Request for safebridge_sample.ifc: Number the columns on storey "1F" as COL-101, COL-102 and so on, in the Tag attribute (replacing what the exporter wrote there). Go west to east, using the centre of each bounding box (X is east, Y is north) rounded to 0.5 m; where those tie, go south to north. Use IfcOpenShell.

First a look at what the model holds.

```python
import ifcopenshell
import ifcopenshell.util.element
import ifcopenshell.util.placement

model = ifcopenshell.open("safebridge_sample.ifc")
print(model.schema)
storey = next(s for s in model.by_type("IfcBuildingStorey") if s.Name == "1F")
columns = [e for e in ifcopenshell.util.element.get_decomposition(storey) if e.is_a("IfcColumn")]
for e in sorted(columns, key=lambda e: e.id()):
    origin = ifcopenshell.util.placement.get_local_placement(e.ObjectPlacement)[:3, 3]
    print(e.id(), e.Tag, e.Name, origin.round(2) + 0.0, sep=" | ")
```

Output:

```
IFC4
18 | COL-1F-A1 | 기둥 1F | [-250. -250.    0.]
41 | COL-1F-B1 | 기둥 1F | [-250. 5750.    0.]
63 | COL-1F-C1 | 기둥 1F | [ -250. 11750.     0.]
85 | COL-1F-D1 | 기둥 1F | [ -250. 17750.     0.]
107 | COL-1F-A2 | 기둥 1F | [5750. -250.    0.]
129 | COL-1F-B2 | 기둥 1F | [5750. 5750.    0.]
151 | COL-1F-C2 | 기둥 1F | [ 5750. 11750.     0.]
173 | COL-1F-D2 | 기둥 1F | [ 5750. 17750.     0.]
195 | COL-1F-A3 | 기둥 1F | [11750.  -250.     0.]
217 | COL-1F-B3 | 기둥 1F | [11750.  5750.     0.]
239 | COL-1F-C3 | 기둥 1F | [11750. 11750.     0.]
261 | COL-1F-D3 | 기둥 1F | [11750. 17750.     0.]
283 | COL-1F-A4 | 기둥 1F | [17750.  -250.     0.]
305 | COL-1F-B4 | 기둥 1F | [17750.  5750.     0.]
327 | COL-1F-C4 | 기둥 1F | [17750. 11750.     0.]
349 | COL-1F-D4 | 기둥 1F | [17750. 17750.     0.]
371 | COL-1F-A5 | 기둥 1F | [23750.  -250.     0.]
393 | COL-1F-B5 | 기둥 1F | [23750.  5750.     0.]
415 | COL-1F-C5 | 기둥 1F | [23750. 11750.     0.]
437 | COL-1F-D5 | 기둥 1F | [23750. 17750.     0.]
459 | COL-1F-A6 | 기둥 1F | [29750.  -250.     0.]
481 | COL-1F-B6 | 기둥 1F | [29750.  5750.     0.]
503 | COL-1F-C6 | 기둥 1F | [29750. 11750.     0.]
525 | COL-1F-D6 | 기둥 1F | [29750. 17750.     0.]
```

```python
import ifcopenshell
import ifcopenshell.geom
import ifcopenshell.util.element
import ifcopenshell.util.shape

model = ifcopenshell.open("safebridge_sample.ifc")
settings = ifcopenshell.geom.settings()
settings.set("use-world-coords", True)


def centre(element):
    shape = ifcopenshell.geom.create_shape(settings, element)
    return ifcopenshell.util.shape.get_bbox_centroid(shape.geometry)


storey = next(s for s in model.by_type("IfcBuildingStorey") if s.Name == "1F")
columns = [e for e in ifcopenshell.util.element.get_decomposition(storey) if e.is_a("IfcColumn")]

# Insertion points can sit at a corner or the storey origin, so sort by the geometry (in metres).
centres = {e: centre(e) for e in columns}
columns.sort(key=lambda e: (round(centres[e][0] / 0.5), centres[e][1]))

for i, e in enumerate(columns, start=1):
    number = f"COL-1{i:02d}"
    e.Tag = number
    print(e.id(), number)

model.write("safebridge_sample_v2.ifc")
```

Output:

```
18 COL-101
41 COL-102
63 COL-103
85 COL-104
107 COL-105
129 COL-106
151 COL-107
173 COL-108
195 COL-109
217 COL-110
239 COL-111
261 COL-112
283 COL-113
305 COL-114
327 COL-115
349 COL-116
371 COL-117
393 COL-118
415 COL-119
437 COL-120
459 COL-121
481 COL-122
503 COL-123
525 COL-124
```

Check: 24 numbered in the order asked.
